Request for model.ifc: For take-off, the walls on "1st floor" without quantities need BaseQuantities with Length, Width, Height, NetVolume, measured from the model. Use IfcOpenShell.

First a look at what the model holds.

```python
import ifcopenshell
import ifcopenshell.util.element
import ifcopenshell.util.unit

model = ifcopenshell.open("model.ifc")
print(model.schema)
for unit_type in ("LENGTHUNIT", "AREAUNIT", "VOLUMEUNIT"):
    print(unit_type, ifcopenshell.util.unit.calculate_unit_scale(model, unit_type))
storey = next(s for s in model.by_type("IfcBuildingStorey") if s.Name == "1st floor")
walls = [e for e in ifcopenshell.util.element.get_decomposition(storey) if e.is_a("IfcWall")]
for e in sorted(walls, key=lambda e: e.id()):
    print(e.id(), e.is_a(), e.Name, list(ifcopenshell.util.element.get_psets(e, qtos_only=True)), sep=" | ")
```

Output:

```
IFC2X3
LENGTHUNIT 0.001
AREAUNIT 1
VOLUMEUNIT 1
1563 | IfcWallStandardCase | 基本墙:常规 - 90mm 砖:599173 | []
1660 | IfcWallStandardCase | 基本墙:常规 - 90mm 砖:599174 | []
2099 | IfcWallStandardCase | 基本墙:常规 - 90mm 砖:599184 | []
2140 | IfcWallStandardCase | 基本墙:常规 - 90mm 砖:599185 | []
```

```python
import ifcopenshell
import ifcopenshell.api.pset
import ifcopenshell.geom
import ifcopenshell.util.element
import ifcopenshell.util.shape
import ifcopenshell.util.unit

model = ifcopenshell.open("model.ifc")
unit_scale = ifcopenshell.util.unit.calculate_unit_scale(model)
volume_scale = ifcopenshell.util.unit.calculate_unit_scale(model, "VOLUMEUNIT")
settings = ifcopenshell.geom.settings()

storey = next(s for s in model.by_type("IfcBuildingStorey") if s.Name == "1st floor")
walls = [e for e in ifcopenshell.util.element.get_decomposition(storey) if e.is_a("IfcWall")]

for e in sorted(walls, key=lambda e: e.id()):
    if ifcopenshell.util.element.get_psets(e, qtos_only=True, should_inherit=False):
        continue
    # Geometry comes back in metres, in the element's own axes.
    shape = ifcopenshell.geom.create_shape(settings, e)
    values = {
        "Length": ifcopenshell.util.shape.get_x(shape.geometry) / unit_scale,
        "Width": ifcopenshell.util.shape.get_y(shape.geometry) / unit_scale,
        "Height": ifcopenshell.util.shape.get_z(shape.geometry) / unit_scale,
        "NetVolume": ifcopenshell.util.shape.get_volume(shape.geometry) / volume_scale,
    }
    qto = ifcopenshell.api.pset.add_qto(model, product=e, name="BaseQuantities")
    ifcopenshell.api.pset.edit_qto(model, qto=qto, properties=values)
    print(e.id(), {k: round(v, 3) for k, v in values.items()})

model.write("model_v2.ifc")
```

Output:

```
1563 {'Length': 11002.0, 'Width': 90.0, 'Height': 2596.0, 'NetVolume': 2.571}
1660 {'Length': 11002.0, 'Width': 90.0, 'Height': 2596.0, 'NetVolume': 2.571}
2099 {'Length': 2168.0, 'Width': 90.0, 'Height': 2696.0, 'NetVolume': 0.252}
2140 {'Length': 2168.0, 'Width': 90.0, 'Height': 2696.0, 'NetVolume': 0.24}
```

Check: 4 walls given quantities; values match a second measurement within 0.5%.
